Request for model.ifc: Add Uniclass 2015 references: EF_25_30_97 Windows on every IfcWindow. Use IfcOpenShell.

First a look at what the model holds.

```python
import ifcopenshell

model = ifcopenshell.open("model.ifc")
print(model.schema)
print("classifications:", [c.Name for c in model.by_type("IfcClassification")])
for ifc_class in ("IfcDoor", "IfcRoof", "IfcStair", "IfcWall", "IfcWindow"):
    print(ifc_class, len(model.by_type(ifc_class)))
```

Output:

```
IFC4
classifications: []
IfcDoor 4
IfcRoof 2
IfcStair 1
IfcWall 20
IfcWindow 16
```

```python
import ifcopenshell
import ifcopenshell.api.classification

model = ifcopenshell.open("model.ifc")

system = ifcopenshell.api.classification.add_classification(model, classification="Uniclass 2015")

codes = {
    "IfcWindow": ("EF_25_30_97", "Windows"),
}
for ifc_class, (code, name) in codes.items():
    products = model.by_type(ifc_class)
    ifcopenshell.api.classification.add_reference(
        model, products=products, classification=system, identification=code, name=name
    )
    print(code, len(products))

model.write("model-out.ifc")
```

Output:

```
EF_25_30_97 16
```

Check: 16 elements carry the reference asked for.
